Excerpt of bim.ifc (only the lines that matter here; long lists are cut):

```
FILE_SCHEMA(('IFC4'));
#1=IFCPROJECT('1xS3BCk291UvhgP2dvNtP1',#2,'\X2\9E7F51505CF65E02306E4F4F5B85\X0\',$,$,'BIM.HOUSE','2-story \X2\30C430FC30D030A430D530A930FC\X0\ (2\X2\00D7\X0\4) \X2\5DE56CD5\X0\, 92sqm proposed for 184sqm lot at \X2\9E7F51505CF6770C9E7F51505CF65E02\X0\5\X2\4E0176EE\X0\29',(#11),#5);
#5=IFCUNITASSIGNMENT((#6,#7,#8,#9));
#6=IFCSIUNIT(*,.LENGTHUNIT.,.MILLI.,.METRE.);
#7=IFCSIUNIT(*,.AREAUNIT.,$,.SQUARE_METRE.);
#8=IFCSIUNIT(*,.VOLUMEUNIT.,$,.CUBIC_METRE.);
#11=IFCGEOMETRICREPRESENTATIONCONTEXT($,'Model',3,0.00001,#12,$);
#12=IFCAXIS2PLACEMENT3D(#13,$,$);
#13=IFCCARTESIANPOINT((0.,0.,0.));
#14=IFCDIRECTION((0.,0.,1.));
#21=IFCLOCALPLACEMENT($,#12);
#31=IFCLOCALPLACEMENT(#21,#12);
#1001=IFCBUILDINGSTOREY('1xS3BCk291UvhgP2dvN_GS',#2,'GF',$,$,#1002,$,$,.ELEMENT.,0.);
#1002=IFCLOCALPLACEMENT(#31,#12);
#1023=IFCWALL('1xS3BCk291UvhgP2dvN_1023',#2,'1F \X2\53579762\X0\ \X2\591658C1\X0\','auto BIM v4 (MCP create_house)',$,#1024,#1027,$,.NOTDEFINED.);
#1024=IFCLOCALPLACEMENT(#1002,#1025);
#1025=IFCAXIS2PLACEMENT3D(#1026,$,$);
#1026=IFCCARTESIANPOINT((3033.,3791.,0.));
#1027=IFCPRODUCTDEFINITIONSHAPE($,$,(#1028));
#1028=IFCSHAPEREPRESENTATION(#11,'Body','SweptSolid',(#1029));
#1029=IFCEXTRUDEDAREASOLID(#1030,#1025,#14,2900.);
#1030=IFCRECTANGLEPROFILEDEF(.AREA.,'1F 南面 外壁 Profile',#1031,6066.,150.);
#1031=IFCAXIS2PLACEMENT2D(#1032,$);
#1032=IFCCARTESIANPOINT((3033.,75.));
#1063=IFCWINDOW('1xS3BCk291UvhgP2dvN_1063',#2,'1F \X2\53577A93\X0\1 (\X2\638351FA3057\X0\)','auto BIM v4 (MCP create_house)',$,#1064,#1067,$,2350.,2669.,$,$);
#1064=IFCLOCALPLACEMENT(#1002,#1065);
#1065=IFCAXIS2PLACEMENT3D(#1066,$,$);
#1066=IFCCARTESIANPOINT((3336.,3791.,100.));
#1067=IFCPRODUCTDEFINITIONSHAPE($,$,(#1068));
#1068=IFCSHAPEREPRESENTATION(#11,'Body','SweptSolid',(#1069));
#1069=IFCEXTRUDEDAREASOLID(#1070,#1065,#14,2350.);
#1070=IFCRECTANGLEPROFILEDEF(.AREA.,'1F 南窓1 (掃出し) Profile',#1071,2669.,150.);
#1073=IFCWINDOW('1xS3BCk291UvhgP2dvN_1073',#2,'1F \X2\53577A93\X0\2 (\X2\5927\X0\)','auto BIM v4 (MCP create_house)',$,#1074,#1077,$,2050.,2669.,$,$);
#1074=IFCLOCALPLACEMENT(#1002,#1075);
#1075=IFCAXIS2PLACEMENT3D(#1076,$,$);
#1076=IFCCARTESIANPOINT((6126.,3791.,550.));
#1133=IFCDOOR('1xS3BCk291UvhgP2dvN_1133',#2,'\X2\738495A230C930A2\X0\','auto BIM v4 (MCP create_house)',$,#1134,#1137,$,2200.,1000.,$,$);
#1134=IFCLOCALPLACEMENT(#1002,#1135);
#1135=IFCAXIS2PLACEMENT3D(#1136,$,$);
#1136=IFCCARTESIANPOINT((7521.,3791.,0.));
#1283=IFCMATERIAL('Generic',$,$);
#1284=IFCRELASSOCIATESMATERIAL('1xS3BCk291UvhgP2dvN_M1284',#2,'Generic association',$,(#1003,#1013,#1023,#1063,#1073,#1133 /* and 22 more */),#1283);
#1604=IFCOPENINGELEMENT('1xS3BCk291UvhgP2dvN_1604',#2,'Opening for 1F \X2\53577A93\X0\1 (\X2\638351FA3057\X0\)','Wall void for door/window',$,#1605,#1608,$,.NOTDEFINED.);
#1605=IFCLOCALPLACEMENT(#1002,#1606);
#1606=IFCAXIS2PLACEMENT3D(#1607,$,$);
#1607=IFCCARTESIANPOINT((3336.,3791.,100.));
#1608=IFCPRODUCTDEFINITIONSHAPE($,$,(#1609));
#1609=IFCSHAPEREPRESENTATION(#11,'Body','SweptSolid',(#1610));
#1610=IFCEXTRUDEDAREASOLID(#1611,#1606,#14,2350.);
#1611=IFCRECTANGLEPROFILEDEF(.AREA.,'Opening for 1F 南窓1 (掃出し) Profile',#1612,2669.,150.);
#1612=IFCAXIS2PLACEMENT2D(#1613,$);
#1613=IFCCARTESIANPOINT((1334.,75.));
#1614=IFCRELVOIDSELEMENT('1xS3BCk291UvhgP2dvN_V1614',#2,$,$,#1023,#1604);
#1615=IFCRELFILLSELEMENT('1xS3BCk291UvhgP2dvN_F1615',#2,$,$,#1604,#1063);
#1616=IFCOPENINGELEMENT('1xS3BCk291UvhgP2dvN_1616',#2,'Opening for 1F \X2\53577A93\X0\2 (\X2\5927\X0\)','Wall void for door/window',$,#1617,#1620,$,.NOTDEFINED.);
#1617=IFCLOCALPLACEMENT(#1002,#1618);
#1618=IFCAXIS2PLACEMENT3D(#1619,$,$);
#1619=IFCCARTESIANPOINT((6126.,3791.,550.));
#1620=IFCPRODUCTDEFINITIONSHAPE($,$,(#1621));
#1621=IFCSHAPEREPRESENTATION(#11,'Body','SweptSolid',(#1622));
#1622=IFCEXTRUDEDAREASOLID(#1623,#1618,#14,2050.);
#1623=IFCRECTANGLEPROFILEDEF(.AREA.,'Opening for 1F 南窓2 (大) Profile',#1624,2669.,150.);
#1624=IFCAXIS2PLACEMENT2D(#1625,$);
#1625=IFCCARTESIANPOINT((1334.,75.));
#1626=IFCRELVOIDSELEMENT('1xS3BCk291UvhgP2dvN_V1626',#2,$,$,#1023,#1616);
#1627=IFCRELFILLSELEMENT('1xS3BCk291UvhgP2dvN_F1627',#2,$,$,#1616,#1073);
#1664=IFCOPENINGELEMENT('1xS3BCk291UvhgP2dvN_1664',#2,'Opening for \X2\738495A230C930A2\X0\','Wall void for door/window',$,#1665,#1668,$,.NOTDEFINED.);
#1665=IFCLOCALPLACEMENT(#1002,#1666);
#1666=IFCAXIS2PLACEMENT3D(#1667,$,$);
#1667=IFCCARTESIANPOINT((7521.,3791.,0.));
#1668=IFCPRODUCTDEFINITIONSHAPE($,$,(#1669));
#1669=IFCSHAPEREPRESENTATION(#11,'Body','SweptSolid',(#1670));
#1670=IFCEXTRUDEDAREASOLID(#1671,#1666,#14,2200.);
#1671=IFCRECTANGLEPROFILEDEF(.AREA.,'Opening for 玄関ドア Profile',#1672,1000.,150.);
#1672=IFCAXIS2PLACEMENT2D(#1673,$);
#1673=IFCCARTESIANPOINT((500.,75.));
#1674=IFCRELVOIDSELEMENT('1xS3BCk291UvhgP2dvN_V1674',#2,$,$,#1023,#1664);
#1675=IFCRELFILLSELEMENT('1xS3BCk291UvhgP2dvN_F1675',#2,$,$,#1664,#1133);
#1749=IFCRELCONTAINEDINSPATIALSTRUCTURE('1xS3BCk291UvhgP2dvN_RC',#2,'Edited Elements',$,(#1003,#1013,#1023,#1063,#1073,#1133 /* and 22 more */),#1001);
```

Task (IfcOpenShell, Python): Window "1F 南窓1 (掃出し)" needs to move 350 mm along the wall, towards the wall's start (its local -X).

```python
import ifcopenshell
import ifcopenshell.api.geometry
import ifcopenshell.util.placement

model = ifcopenshell.open("bim.ifc")

window = model.by_guid("1xS3BCk291UvhgP2dvN_1063")
opening = window.FillsVoids[0].RelatingOpeningElement
wall = opening.VoidsElements[0].RelatingBuildingElement

wall_matrix = ifcopenshell.util.placement.get_local_placement(wall.ObjectPlacement)
shift = wall_matrix[:3, 0] * -350.0
before = ifcopenshell.util.placement.get_local_placement(window.ObjectPlacement)[:3, 3].copy()

# The window is not placed relative to its opening, so move both.
for product in (opening, window):
    matrix = ifcopenshell.util.placement.get_local_placement(product.ObjectPlacement)
    matrix[:3, 3] += shift
    ifcopenshell.api.geometry.edit_object_placement(model, product=product, matrix=matrix, is_si=False)

after = ifcopenshell.util.placement.get_local_placement(window.ObjectPlacement)[:3, 3]
print("window moved by", (after - before).round(3) + 0.0)

model.write("bim-out.ifc")
```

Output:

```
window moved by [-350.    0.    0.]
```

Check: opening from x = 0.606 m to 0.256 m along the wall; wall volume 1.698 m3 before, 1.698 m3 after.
